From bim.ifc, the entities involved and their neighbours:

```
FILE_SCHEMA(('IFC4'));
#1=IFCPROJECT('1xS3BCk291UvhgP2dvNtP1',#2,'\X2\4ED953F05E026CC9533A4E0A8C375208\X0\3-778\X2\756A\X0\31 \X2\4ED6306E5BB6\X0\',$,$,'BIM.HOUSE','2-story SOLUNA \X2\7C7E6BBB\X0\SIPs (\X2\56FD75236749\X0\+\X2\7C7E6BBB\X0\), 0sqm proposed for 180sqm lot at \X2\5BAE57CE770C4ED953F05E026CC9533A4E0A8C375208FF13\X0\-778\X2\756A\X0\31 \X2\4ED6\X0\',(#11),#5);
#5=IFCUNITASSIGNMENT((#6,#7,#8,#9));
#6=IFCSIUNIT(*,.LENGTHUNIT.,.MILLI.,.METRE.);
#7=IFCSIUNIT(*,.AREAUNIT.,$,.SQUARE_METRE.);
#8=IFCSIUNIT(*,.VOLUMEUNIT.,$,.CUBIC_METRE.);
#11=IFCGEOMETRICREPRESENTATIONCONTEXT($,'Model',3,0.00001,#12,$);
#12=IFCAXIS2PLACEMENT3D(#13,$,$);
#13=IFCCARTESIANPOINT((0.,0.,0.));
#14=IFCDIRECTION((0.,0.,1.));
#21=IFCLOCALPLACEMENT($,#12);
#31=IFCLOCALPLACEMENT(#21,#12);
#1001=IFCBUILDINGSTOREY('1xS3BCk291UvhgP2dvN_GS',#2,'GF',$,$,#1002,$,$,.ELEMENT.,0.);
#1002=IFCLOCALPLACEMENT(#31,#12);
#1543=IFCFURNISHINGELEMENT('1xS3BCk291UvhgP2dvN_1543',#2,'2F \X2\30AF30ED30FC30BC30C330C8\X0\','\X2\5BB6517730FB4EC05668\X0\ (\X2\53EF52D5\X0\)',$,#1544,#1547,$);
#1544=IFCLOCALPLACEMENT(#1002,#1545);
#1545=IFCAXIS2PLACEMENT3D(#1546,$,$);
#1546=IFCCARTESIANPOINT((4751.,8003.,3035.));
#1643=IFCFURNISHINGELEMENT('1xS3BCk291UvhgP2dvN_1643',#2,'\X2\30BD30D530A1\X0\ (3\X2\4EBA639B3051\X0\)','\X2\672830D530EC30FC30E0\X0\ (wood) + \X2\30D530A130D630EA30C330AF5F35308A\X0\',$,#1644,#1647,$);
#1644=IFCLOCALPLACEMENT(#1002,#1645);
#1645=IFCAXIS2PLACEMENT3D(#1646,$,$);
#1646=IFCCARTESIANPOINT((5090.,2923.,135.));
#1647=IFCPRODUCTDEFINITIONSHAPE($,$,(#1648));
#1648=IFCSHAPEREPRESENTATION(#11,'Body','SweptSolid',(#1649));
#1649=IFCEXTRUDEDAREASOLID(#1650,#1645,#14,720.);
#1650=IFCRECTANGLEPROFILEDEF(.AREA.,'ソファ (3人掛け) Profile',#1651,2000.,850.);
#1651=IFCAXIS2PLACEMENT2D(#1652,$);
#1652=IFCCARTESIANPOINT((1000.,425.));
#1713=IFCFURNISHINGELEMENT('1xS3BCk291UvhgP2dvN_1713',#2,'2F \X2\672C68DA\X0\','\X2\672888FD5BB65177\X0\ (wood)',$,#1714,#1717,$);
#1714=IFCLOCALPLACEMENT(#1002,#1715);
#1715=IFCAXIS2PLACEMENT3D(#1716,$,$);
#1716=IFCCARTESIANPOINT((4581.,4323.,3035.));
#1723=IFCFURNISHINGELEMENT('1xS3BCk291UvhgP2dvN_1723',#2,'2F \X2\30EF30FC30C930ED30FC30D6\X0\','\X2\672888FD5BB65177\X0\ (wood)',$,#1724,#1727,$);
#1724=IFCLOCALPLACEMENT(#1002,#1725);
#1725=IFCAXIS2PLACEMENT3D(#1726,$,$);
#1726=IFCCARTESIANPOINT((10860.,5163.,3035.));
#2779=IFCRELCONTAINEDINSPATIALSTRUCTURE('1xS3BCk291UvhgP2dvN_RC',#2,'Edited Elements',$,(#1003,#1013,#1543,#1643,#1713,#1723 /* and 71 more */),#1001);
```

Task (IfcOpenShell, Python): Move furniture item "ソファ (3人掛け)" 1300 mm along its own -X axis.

```python
import ifcopenshell
import ifcopenshell.api.geometry
import ifcopenshell.util.placement

model = ifcopenshell.open("bim.ifc")

item = model.by_guid("1xS3BCk291UvhgP2dvN_1643")
matrix = ifcopenshell.util.placement.get_local_placement(item.ObjectPlacement)
matrix[:3, 3] -= matrix[:3, 0] * 1300.0
ifcopenshell.api.geometry.edit_object_placement(model, product=item, matrix=matrix, is_si=False)

print(ifcopenshell.util.placement.get_local_placement(item.ObjectPlacement).round(3) + 0.0)

model.write("bim_rev.ifc")
```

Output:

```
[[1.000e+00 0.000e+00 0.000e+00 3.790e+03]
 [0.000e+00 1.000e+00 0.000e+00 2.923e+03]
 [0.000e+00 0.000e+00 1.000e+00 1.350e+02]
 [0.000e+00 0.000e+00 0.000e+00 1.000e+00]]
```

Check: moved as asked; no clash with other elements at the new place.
